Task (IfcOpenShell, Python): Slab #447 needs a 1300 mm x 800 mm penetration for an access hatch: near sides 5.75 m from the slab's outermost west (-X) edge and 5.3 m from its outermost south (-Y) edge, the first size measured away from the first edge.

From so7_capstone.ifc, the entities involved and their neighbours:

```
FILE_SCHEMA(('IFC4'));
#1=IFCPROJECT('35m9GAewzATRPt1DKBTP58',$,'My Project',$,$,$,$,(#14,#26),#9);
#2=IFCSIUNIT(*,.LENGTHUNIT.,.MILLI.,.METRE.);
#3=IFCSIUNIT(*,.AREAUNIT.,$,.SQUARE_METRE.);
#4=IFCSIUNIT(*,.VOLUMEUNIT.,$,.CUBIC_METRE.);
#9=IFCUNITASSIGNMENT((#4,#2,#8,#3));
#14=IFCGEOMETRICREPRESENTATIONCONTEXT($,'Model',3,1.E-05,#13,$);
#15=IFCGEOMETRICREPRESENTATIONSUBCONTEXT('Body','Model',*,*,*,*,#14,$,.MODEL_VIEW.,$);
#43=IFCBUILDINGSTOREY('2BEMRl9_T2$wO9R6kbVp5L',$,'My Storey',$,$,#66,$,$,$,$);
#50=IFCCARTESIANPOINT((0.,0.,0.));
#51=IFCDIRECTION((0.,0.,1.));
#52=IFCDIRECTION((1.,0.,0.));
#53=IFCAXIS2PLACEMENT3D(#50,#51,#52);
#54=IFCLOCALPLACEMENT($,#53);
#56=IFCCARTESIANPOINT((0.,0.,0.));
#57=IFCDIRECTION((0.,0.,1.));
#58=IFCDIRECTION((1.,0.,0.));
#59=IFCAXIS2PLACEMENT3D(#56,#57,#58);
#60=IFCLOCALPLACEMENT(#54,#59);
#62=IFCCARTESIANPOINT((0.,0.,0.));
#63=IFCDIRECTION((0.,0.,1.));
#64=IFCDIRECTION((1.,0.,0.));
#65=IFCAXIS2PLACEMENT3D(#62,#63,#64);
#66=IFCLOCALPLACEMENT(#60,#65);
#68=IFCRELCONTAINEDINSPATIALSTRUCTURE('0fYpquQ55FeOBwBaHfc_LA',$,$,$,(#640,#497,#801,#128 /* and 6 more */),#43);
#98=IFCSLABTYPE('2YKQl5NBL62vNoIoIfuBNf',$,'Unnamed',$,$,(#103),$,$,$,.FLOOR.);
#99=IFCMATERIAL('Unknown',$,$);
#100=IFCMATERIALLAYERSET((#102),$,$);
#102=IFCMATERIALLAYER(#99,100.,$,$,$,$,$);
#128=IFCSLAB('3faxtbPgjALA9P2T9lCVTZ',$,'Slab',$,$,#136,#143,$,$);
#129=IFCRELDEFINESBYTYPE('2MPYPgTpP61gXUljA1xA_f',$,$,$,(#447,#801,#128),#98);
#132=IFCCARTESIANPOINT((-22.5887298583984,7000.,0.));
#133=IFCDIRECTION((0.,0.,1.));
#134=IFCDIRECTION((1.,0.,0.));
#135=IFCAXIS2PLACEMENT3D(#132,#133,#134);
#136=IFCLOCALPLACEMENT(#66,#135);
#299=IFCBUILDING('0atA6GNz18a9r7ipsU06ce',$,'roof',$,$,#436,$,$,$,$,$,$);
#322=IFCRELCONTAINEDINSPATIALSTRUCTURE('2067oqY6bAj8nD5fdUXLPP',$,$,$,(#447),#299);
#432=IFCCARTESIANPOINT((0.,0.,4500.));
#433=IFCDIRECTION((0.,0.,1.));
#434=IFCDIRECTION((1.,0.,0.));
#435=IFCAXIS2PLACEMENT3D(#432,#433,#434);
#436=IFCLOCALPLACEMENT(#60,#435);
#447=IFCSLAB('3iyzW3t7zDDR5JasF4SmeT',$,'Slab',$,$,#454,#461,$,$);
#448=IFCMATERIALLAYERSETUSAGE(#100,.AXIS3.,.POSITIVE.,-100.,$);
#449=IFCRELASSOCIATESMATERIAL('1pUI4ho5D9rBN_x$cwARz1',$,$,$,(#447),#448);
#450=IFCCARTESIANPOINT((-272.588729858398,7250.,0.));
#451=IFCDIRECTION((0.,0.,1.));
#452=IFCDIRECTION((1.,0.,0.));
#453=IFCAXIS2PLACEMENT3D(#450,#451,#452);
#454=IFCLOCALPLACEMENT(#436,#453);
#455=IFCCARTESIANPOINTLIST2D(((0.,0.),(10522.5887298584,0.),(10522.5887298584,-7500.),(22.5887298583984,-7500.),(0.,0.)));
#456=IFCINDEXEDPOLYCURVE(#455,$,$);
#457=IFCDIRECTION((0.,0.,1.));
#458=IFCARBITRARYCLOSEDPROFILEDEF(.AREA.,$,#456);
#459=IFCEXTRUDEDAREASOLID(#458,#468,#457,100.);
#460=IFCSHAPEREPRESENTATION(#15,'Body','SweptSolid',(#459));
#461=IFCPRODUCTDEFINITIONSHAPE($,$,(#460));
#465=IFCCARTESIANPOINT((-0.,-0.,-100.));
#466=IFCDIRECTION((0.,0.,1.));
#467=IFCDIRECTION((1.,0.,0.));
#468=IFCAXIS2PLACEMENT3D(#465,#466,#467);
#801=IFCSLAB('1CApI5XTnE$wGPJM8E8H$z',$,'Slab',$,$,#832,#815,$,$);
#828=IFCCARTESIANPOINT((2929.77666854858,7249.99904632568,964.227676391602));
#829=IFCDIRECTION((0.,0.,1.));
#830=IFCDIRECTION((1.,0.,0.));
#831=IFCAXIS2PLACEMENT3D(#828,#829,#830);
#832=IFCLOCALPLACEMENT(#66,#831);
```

```python
import numpy as np
import ifcopenshell
import ifcopenshell.api.feature
import ifcopenshell.api.geometry
import ifcopenshell.api.root
import ifcopenshell.geom
import ifcopenshell.util.placement
import ifcopenshell.util.representation
import ifcopenshell.util.shape
import ifcopenshell.util.unit

model = ifcopenshell.open("so7_capstone.ifc")
unit_scale = ifcopenshell.util.unit.calculate_unit_scale(model)
settings = ifcopenshell.geom.settings()


def volume(element):
    """Net volume in cubic metres, openings subtracted."""
    shape = ifcopenshell.geom.create_shape(settings, element)
    return ifcopenshell.util.shape.get_volume(shape.geometry)


slab = model.by_guid("3iyzW3t7zDDR5JasF4SmeT")
before = volume(slab)

# Extent in the slab's own axes, in metres. The edges named are its -X and -Y sides.
slab_shape = ifcopenshell.geom.create_shape(settings, slab)
vertices = ifcopenshell.util.shape.get_vertices(slab_shape.geometry)
x_min, y_min, bottom = vertices.min(axis=0)
top = vertices[:, 2].max()

opening = ifcopenshell.api.root.create_entity(model, ifc_class="IfcOpeningElement", name="Access hatch opening", predefined_type="OPENING")
context = ifcopenshell.util.representation.get_context(model, "Model", "Body", "MODEL_VIEW")
width, depth = 1.3, 0.8
outline = [(0.0, 0.0), (width, 0.0), (width, depth), (0.0, depth), (0.0, 0.0)]
# Overshoot both faces by 50 mm so the cut is clean.
shape = ifcopenshell.api.geometry.add_slab_representation(
    model, context=context, depth=top - bottom + 0.1, polyline=outline
)
ifcopenshell.api.geometry.assign_representation(model, product=opening, representation=shape)

matrix = ifcopenshell.util.placement.get_local_placement(slab.ObjectPlacement)
matrix[:, 3] = matrix @ np.append(np.array([x_min + 5.75, y_min + 5.3, bottom - 0.05]) / unit_scale, 1.0)
ifcopenshell.api.geometry.edit_object_placement(model, product=opening, matrix=matrix, is_si=False)
ifcopenshell.api.feature.add_feature(model, feature=opening, element=slab)

after = volume(slab)

print(f"slab volume {before:.3f} -> {after:.3f} m3")

model.write("so7_capstone_v2.ifc")
```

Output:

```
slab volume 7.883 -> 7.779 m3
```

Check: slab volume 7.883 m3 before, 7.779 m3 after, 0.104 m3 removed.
